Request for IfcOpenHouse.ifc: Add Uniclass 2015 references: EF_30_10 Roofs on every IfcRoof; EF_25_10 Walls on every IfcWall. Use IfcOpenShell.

First a look at what the model holds.

```python
import ifcopenshell

model = ifcopenshell.open("IfcOpenHouse.ifc")
print(model.schema)
print("classifications:", [c.Name for c in model.by_type("IfcClassification")])
for ifc_class in ("IfcDoor", "IfcRoof", "IfcStair", "IfcWall", "IfcWindow"):
    print(ifc_class, len(model.by_type(ifc_class)))
```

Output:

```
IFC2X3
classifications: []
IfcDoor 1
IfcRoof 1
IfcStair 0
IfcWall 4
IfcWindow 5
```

```python
import ifcopenshell
import ifcopenshell.api.classification

model = ifcopenshell.open("IfcOpenHouse.ifc")

# IFC2X3 requires Source and Edition and has no link from the project to the system.
system = model.create_entity("IfcClassification", Source="NBS", Edition="2015", Name="Uniclass 2015")

codes = {
    "IfcRoof": ("EF_30_10", "Roofs"),
    "IfcWall": ("EF_25_10", "Walls"),
}
for ifc_class, (code, name) in codes.items():
    products = model.by_type(ifc_class)
    ifcopenshell.api.classification.add_reference(
        model, products=products, classification=system, identification=code, name=name
    )
    print(code, len(products))

model.write("IfcOpenHouse-out.ifc")
```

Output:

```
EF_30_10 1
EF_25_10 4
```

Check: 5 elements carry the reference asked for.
